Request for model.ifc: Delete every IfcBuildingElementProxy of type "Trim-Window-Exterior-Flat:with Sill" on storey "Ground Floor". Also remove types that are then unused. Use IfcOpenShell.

First a look at what the model holds.

```python
import ifcopenshell
import ifcopenshell.util.element

model = ifcopenshell.open("model.ifc")
print(model.schema)
storey = next(s for s in model.by_type("IfcBuildingStorey") if s.Name == "Ground Floor")
proxies = [e for e in ifcopenshell.util.element.get_decomposition(storey) if e.is_a("IfcBuildingElementProxy")]
seen = {}
for e in proxies:
    element_type = ifcopenshell.util.element.get_type(e)
    name = element_type.Name if element_type not in (None, e) else None
    seen[name] = seen.get(name, 0) + 1
for name, count in sorted(seen.items(), key=str):
    print(count, "x", name)
```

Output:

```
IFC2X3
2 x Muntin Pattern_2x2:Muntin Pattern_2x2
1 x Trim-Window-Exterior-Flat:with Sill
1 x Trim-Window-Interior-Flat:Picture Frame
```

```python
import ifcopenshell
import ifcopenshell.api.root
import ifcopenshell.util.element

model = ifcopenshell.open("model.ifc")

storey = next(s for s in model.by_type("IfcBuildingStorey") if s.Name == "Ground Floor")
proxies = [e for e in ifcopenshell.util.element.get_decomposition(storey) if e.is_a("IfcBuildingElementProxy")]
targets = [e for e in proxies if (t := ifcopenshell.util.element.get_type(e)) not in (None, e) and t.Name == "Trim-Window-Exterior-Flat:with Sill"]
types = {ifcopenshell.util.element.get_type(e) for e in targets} - {None, *targets}

for e in targets:
    ifcopenshell.api.root.remove_product(model, product=e)
print(len(targets), "removed")

unused = [t for t in types if not ifcopenshell.util.element.get_types(t)]
for t in unused:
    ifcopenshell.api.root.remove_product(model, product=t)
print(len(unused), "unused types removed")

model.write("model-out.ifc")
```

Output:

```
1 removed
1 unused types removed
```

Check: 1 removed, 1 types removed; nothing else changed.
